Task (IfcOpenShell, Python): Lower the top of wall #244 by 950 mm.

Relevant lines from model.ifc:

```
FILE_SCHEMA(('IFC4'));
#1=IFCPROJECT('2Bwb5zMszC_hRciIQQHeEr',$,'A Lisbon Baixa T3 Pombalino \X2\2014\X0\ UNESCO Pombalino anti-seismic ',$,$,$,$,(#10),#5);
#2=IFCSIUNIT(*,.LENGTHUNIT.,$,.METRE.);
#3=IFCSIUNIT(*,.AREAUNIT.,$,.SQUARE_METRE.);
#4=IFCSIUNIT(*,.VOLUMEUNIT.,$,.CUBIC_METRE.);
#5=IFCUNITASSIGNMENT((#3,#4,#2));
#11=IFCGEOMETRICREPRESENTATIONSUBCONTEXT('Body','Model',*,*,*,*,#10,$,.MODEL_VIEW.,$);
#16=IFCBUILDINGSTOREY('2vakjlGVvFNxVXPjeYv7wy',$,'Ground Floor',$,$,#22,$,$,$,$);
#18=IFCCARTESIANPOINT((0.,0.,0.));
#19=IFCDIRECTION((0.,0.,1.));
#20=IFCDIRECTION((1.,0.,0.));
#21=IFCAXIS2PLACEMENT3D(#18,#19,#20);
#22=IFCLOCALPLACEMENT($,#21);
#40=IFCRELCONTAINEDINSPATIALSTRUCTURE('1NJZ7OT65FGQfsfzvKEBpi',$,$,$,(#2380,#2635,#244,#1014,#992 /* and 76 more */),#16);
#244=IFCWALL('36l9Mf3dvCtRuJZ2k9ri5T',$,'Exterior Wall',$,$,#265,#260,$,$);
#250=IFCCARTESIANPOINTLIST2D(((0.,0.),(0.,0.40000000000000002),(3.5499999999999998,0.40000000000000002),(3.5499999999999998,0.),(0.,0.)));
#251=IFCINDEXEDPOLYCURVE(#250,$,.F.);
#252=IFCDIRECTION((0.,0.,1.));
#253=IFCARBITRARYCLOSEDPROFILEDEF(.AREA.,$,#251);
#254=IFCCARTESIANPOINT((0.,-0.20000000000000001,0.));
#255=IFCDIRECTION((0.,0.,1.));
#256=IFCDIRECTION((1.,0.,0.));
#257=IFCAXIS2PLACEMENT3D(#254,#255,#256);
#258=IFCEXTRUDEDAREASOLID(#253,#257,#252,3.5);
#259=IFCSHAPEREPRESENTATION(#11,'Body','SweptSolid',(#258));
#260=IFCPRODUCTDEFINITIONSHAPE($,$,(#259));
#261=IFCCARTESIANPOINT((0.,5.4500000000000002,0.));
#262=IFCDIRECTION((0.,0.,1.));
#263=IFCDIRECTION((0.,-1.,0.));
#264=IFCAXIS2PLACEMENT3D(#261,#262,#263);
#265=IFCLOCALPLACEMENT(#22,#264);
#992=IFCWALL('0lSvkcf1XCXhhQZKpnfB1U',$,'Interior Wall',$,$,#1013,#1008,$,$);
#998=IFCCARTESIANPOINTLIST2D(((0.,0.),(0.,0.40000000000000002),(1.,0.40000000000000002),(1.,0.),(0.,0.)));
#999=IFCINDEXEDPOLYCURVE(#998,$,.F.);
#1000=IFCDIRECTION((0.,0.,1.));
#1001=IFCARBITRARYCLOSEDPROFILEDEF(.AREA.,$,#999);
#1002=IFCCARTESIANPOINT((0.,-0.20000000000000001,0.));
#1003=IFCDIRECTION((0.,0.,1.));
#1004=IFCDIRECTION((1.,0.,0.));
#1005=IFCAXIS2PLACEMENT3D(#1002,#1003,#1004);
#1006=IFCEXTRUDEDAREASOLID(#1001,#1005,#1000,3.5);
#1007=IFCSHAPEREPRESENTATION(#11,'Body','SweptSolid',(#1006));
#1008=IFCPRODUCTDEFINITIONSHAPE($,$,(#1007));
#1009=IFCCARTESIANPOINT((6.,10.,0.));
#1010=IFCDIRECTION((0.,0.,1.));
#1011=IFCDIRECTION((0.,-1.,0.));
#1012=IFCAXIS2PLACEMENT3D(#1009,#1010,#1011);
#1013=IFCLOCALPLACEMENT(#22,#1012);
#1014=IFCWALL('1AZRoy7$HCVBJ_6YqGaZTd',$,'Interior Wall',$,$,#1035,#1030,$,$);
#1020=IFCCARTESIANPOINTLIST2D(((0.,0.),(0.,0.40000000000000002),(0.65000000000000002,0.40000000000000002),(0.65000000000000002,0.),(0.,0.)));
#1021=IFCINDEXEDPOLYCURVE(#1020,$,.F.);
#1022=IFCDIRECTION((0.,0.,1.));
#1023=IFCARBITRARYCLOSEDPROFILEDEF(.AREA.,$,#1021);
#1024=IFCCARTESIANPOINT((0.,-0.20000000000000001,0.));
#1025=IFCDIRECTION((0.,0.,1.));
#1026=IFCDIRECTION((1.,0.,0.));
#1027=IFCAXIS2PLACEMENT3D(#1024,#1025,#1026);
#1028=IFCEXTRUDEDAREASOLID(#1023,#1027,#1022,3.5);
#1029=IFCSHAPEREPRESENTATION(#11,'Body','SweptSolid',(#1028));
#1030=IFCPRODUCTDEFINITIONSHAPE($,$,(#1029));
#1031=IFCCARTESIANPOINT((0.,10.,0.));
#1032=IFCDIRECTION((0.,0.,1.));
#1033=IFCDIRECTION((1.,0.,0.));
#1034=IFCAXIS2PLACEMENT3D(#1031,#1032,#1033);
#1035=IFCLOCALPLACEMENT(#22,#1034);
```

```python
import ifcopenshell
import ifcopenshell.geom
import ifcopenshell.util.representation
import ifcopenshell.util.shape
import ifcopenshell.util.unit

model = ifcopenshell.open("model.ifc")
unit_scale = ifcopenshell.util.unit.calculate_unit_scale(model)
settings = ifcopenshell.geom.settings()


def volume(element):
    """Net volume in cubic metres, openings subtracted."""
    shape = ifcopenshell.geom.create_shape(settings, element)
    return ifcopenshell.util.shape.get_volume(shape.geometry)


wall = model.by_guid("36l9Mf3dvCtRuJZ2k9ri5T")
before = volume(wall)

body = ifcopenshell.util.representation.get_representation(wall, "Model", "Body")
solid = body.Items[0]
old_height = solid.Depth
solid.Depth -= 0.95 / unit_scale
after = volume(wall)

print(f"height {old_height:g} -> {solid.Depth:g}, volume {before:.3f} -> {after:.3f} m3")

model.write("model_rev.ifc")
```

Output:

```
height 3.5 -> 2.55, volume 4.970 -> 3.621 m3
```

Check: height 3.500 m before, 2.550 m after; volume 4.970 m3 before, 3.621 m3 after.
